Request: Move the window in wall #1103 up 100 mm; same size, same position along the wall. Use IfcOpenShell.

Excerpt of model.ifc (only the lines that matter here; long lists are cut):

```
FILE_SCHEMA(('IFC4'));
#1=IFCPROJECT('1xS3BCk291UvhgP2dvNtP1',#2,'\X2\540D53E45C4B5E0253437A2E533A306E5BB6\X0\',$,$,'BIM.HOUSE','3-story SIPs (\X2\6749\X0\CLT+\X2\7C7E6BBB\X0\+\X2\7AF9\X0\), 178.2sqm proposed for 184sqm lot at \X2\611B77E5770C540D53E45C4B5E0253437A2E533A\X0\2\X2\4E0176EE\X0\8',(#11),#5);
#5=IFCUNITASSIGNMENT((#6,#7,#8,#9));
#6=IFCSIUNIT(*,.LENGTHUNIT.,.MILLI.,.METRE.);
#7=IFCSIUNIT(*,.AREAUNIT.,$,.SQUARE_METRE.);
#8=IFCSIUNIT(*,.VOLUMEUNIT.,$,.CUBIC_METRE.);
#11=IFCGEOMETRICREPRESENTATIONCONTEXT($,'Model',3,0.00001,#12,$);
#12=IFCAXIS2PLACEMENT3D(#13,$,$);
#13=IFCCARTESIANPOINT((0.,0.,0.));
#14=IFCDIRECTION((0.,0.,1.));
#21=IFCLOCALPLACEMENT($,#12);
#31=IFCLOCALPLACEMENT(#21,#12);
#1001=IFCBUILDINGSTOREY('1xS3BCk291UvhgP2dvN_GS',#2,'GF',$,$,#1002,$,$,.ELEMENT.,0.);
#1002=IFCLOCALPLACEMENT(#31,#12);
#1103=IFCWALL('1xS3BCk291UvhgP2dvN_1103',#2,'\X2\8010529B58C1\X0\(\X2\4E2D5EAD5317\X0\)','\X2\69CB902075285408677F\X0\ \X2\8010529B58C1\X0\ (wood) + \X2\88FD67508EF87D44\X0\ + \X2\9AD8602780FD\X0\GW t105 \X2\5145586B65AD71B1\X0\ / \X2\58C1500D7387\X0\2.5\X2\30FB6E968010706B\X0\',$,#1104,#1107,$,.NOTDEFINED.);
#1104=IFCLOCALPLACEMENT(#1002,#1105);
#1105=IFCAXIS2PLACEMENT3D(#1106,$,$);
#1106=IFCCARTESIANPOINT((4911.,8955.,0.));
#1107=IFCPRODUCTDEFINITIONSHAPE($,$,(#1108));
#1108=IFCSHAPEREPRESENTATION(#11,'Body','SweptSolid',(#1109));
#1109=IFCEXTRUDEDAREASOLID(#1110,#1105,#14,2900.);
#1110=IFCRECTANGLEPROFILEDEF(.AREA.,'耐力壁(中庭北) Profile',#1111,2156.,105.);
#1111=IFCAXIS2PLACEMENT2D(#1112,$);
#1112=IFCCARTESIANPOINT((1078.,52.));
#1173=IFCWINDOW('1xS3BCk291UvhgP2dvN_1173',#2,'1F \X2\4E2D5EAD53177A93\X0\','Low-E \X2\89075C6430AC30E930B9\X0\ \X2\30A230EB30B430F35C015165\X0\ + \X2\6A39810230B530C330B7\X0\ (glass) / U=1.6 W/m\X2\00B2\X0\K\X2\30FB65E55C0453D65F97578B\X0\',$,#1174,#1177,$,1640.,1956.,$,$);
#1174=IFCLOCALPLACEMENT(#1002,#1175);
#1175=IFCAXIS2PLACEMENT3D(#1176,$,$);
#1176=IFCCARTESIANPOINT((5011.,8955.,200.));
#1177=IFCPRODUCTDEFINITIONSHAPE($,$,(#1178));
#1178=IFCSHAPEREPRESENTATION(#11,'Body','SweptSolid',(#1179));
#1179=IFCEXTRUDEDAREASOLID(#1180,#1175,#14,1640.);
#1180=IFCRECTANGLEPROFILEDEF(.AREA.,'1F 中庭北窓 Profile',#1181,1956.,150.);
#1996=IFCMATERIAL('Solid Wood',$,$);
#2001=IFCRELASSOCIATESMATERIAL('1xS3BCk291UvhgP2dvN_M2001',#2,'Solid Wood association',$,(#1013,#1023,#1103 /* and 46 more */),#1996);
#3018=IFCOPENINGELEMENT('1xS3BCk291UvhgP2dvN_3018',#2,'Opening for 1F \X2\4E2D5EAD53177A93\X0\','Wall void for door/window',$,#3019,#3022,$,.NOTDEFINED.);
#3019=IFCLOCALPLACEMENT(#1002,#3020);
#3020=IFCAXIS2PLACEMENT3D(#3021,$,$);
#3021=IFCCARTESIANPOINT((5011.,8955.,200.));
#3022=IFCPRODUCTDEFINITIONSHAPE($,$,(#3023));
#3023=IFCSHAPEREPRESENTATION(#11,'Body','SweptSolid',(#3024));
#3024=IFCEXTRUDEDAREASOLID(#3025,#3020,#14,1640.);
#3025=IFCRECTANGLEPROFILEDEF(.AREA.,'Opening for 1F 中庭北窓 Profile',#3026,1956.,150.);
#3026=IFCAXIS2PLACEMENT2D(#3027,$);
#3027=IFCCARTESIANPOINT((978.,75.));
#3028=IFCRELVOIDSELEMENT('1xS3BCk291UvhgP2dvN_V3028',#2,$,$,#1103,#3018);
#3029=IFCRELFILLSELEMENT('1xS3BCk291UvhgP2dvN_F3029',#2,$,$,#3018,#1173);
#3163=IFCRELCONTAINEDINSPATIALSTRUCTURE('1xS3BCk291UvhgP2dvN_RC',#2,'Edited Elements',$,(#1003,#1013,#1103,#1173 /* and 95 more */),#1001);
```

```python
import numpy as np
import ifcopenshell
import ifcopenshell.api.geometry
import ifcopenshell.util.placement
import ifcopenshell.util.unit

model = ifcopenshell.open("model.ifc")
unit_scale = ifcopenshell.util.unit.calculate_unit_scale(model)

window = model.by_guid("1xS3BCk291UvhgP2dvN_1173")
opening = window.FillsVoids[0].RelatingOpeningElement
dz = 100.0

shift = np.array([0.0, 0.0, dz])
# The window is not placed relative to its opening, so move both.
for product in (opening, window):
    matrix = ifcopenshell.util.placement.get_local_placement(product.ObjectPlacement)
    matrix[:3, 3] += shift
    ifcopenshell.api.geometry.edit_object_placement(model, product=product, matrix=matrix, is_si=False)

print(f"moved by {dz * unit_scale:+.3f} m")

model.write("model_edited.ifc")
```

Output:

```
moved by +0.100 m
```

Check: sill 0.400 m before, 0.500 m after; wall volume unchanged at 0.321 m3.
